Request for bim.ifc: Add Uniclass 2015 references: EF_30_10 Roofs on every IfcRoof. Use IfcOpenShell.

First a look at what the model holds.

```python
import ifcopenshell

model = ifcopenshell.open("bim.ifc")
print(model.schema)
print("classifications:", [c.Name for c in model.by_type("IfcClassification")])
for ifc_class in ("IfcDoor", "IfcRoof", "IfcStair", "IfcWall", "IfcWindow"):
    print(ifc_class, len(model.by_type(ifc_class)))
```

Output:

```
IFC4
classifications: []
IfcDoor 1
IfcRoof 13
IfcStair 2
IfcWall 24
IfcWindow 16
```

```python
import ifcopenshell
import ifcopenshell.api.classification

model = ifcopenshell.open("bim.ifc")

system = ifcopenshell.api.classification.add_classification(model, classification="Uniclass 2015")

codes = {
    "IfcRoof": ("EF_30_10", "Roofs"),
}
for ifc_class, (code, name) in codes.items():
    products = model.by_type(ifc_class)
    ifcopenshell.api.classification.add_reference(
        model, products=products, classification=system, identification=code, name=name
    )
    print(code, len(products))

model.write("bim_v2.ifc")
```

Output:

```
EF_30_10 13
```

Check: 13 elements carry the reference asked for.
